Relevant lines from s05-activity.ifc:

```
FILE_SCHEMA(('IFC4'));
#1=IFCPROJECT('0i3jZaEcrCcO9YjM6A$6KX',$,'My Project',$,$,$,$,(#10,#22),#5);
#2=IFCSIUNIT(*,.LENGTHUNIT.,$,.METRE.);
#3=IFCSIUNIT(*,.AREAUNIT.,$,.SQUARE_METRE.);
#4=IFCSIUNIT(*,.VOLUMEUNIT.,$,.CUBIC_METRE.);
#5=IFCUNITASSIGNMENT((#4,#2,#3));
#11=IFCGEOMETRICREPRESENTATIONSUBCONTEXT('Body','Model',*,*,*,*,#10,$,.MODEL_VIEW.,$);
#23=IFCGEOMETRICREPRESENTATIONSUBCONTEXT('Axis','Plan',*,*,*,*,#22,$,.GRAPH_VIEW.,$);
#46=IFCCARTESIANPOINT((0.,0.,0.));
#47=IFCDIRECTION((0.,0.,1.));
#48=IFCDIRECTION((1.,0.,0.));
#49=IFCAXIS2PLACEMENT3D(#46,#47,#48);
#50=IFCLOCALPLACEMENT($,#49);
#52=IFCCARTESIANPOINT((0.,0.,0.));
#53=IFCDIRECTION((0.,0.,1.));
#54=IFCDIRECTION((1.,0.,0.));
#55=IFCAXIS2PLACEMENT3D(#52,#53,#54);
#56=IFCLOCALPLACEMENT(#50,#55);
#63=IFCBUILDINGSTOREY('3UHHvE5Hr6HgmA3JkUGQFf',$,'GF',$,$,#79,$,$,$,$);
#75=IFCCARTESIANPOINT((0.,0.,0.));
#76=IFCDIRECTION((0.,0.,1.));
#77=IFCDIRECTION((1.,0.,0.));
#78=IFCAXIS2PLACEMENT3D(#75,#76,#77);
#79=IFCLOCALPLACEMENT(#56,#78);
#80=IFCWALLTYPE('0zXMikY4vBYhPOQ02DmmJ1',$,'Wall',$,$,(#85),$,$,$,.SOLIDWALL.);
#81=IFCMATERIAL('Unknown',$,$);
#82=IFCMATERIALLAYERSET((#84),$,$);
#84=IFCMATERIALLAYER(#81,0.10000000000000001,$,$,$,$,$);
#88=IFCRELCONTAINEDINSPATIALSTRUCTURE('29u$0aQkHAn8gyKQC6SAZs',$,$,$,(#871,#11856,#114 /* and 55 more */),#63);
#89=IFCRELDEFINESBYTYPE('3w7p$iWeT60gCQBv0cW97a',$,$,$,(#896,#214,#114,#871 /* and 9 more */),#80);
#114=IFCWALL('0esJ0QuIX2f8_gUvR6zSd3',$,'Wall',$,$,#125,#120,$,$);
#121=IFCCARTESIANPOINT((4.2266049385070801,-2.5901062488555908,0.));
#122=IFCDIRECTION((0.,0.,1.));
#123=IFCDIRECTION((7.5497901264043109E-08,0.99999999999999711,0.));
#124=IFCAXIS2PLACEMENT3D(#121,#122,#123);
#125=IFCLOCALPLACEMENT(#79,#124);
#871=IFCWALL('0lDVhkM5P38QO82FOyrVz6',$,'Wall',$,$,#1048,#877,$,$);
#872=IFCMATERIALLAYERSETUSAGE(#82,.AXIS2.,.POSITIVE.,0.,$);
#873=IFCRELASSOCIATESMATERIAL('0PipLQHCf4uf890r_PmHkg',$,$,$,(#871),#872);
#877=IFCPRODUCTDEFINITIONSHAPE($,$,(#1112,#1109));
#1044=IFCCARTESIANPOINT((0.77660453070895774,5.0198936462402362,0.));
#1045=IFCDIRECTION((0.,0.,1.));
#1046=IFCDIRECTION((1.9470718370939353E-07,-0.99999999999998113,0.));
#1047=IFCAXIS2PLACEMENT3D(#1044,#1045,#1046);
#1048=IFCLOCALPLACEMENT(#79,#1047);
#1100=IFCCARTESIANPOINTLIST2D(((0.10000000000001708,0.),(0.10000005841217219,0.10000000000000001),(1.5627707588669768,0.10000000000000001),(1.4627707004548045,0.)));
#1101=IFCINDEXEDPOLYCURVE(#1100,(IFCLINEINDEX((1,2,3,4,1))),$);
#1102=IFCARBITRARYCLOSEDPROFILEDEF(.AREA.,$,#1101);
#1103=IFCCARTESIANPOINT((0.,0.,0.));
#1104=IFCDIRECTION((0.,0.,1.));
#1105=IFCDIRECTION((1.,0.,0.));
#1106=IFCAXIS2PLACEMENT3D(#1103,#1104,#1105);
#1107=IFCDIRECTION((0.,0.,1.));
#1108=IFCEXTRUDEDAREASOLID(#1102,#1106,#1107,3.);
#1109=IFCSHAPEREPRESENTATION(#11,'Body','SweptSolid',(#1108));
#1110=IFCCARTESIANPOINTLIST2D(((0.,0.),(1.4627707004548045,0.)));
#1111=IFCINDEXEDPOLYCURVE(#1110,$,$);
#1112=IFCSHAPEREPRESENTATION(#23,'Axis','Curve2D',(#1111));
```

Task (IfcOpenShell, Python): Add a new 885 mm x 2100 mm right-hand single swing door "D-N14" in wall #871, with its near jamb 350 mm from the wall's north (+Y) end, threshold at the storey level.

```python
import numpy as np
import ifcopenshell
import ifcopenshell.api.feature
import ifcopenshell.api.geometry
import ifcopenshell.api.root
import ifcopenshell.api.spatial
import ifcopenshell.geom
import ifcopenshell.util.element
import ifcopenshell.util.placement
import ifcopenshell.util.representation
import ifcopenshell.util.shape
import ifcopenshell.util.unit

model = ifcopenshell.open("s05-activity.ifc")
unit_scale = ifcopenshell.util.unit.calculate_unit_scale(model)
settings = ifcopenshell.geom.settings()


def volume(element):
    """Net volume in cubic metres, openings subtracted."""
    shape = ifcopenshell.geom.create_shape(settings, element)
    return ifcopenshell.util.shape.get_volume(shape.geometry)


wall = model.by_guid("0lDVhkM5P38QO82FOyrVz6")
storey = ifcopenshell.util.element.get_container(wall, ifc_class="IfcBuildingStorey")
context = ifcopenshell.util.representation.get_context(model, "Model", "Body", "MODEL_VIEW")
before = volume(wall)

width, height, from_end, sill = 0.885, 2.1, 0.35, 0.0  # metres

# The wall runs along its own X axis, and the end named is its -X end.
wall_shape = ifcopenshell.geom.create_shape(settings, wall)
x, y, z = ifcopenshell.util.shape.get_vertices(wall_shape.geometry).T
start = x.min() + from_end
face, thickness = float(y.min()), float(y.max() - y.min())
wall_matrix = ifcopenshell.util.placement.get_local_placement(wall.ObjectPlacement)
level = ifcopenshell.util.placement.get_local_placement(storey.ObjectPlacement)[2, 3]


def in_wall(x, y):
    """Placement at x, y metres in the wall's axes, at sill height."""
    matrix = wall_matrix.copy()
    matrix[:, 3] = wall_matrix @ np.array([x / unit_scale, y / unit_scale, 0.0, 1.0])
    matrix[2, 3] = level + sill / unit_scale
    return matrix


# Opening: a box that overshoots both wall faces by 50 mm.
opening = ifcopenshell.api.root.create_entity(model, ifc_class="IfcOpeningElement", predefined_type="OPENING")
box = ifcopenshell.api.geometry.add_wall_representation(
    model, context=context, length=width, height=height, thickness=thickness + 0.1
)
ifcopenshell.api.geometry.assign_representation(model, product=opening, representation=box)
ifcopenshell.api.geometry.edit_object_placement(model, product=opening, matrix=in_wall(start, face - 0.05), is_si=False)
ifcopenshell.api.feature.add_feature(model, feature=opening, element=wall)

door = ifcopenshell.api.root.create_entity(model, ifc_class="IfcDoor", name="D-N14", predefined_type="DOOR")
door.OverallWidth, door.OverallHeight = width / unit_scale, height / unit_scale
door.OperationType = "SINGLE_SWING_RIGHT"
body = ifcopenshell.api.geometry.add_door_representation(
    model,
    context=context,
    overall_width=door.OverallWidth,
    overall_height=door.OverallHeight,
    operation_type="SINGLE_SWING_RIGHT",
    lining_properties={"LiningDepth": thickness / unit_scale, "ThresholdDepth": thickness / unit_scale},
)
ifcopenshell.api.geometry.assign_representation(model, product=door, representation=body)
ifcopenshell.api.spatial.assign_container(model, products=[door], relating_structure=storey)
ifcopenshell.api.feature.add_filling(model, opening=opening, element=door)

# The lining spans the wall, so the door starts at the wall face.
ifcopenshell.api.geometry.edit_object_placement(model, product=door, matrix=in_wall(start, face), is_si=False)

after = volume(wall)

print(f"wall volume {before:.3f} -> {after:.3f} m3")

model.write("s05-activity_rev.ifc")
```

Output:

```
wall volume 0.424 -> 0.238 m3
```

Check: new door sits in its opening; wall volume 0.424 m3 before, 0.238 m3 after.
